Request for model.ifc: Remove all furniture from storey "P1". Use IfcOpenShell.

First a look at what the model holds.

```python
import ifcopenshell
import ifcopenshell.util.element

model = ifcopenshell.open("model.ifc")
print(model.schema)
storey = next(s for s in model.by_type("IfcBuildingStorey") if s.Name == "P1")
furniture = [e for e in ifcopenshell.util.element.get_decomposition(storey) if e.is_a("IfcFurnishingElement")]
seen = {}
for e in furniture:
    element_type = ifcopenshell.util.element.get_type(e)
    name = element_type.Name if element_type not in (None, e) else None
    seen[name] = seen.get(name, 0) + 1
for name, count in sorted(seen.items(), key=str):
    print(count, "x", name)
```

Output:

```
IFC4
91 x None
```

```python
import ifcopenshell
import ifcopenshell.api.root
import ifcopenshell.util.element

model = ifcopenshell.open("model.ifc")

storey = next(s for s in model.by_type("IfcBuildingStorey") if s.Name == "P1")
furniture = [e for e in ifcopenshell.util.element.get_decomposition(storey) if e.is_a("IfcFurnishingElement")]

for e in furniture:
    ifcopenshell.api.root.remove_product(model, product=e)
print(len(furniture), "removed")

model.write("model_rev.ifc")
```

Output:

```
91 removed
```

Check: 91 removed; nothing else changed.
